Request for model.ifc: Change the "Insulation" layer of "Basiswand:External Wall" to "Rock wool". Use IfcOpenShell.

First a look at what the model holds.

```python
import ifcopenshell
import ifcopenshell.util.element

model = ifcopenshell.open("model.ifc")
print(model.schema)
for layer_set in model.by_type("IfcMaterialLayerSet"):
    if layer_set.LayerSetName == "Basiswand:External Wall":
        for layer in layer_set.MaterialLayers:
            print(layer.id(), layer.Material and layer.Material.Name, layer.LayerThickness, sep=" | ")
        print(len(ifcopenshell.util.element.get_elements_by_material(model, layer_set)), "elements and types use it")
print(sorted(m.Name for m in model.by_type("IfcMaterial") if m.Name)[:60])
```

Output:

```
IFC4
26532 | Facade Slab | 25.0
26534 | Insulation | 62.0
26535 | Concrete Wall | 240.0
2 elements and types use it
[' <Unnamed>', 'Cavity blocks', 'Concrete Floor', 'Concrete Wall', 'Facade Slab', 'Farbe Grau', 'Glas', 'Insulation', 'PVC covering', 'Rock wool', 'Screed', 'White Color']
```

```python
import ifcopenshell
import ifcopenshell.api.material

model = ifcopenshell.open("model.ifc")

layer_set = next(s for s in model.by_type("IfcMaterialLayerSet") if s.LayerSetName == "Basiswand:External Wall")
layer = next(l for l in layer_set.MaterialLayers if l.Material and l.Material.Name == "Insulation")
material = next(m for m in model.by_type("IfcMaterial") if m.Name == "Rock wool")

# Point this one layer at the other material; renaming the old one would change it everywhere.
ifcopenshell.api.material.edit_layer(model, layer=layer, attributes={}, material=material)

print([l.Material.Name if l.Material else None for l in layer_set.MaterialLayers])

model.write("model_rev.ifc")
```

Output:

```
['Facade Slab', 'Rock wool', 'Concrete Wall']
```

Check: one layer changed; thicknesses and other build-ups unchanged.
